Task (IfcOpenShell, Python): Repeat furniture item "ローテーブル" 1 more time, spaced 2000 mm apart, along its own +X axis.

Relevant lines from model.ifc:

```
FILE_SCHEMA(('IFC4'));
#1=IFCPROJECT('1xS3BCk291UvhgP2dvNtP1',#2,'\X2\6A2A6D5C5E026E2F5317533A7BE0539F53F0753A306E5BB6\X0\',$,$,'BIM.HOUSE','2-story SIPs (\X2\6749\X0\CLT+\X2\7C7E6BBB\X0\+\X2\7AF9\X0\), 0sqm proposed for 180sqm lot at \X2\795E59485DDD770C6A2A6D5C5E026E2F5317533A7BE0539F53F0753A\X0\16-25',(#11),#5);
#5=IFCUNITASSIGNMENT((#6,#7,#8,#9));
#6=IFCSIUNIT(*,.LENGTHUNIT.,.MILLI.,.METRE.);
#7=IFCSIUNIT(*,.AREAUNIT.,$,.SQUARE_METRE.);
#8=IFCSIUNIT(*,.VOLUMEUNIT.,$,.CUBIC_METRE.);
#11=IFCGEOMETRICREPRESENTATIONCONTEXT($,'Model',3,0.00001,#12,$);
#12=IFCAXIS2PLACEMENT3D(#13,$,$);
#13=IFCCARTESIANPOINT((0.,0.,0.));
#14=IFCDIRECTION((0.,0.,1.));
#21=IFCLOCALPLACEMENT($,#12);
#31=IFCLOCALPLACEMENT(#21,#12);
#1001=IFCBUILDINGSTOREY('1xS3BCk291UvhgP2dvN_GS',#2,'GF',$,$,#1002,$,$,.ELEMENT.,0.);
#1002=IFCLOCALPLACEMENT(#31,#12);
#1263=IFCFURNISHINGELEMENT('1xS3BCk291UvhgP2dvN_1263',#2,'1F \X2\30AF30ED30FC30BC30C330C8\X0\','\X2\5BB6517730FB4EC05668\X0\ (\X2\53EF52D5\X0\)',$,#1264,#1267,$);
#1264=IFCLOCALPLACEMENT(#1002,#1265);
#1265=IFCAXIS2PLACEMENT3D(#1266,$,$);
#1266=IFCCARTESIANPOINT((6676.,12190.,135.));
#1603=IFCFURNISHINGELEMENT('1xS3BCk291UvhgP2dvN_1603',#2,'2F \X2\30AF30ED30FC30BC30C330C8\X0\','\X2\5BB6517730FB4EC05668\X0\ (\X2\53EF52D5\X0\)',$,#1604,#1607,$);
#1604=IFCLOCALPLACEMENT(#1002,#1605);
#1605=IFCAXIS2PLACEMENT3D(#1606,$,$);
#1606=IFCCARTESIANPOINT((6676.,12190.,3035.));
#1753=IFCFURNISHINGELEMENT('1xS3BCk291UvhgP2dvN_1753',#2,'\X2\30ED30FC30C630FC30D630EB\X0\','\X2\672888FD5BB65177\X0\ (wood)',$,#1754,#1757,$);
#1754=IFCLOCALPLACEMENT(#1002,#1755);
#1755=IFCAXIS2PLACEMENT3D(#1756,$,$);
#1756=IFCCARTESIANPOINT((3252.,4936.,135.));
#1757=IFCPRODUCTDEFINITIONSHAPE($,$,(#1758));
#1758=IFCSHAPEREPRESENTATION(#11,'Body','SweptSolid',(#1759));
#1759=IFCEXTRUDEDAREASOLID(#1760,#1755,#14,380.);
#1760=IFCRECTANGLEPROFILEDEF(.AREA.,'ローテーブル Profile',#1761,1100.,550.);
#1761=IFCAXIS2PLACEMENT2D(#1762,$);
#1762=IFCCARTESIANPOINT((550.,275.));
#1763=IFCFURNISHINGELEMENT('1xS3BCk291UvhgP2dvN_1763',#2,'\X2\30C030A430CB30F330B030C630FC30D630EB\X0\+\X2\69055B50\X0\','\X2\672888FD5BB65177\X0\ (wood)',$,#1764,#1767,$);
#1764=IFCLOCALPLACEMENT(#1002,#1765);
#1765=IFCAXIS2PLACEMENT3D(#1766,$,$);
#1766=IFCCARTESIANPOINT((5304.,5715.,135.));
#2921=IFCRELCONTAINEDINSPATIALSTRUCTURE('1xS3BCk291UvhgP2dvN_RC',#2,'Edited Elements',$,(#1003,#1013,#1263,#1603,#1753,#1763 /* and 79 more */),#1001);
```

```python
import ifcopenshell
import ifcopenshell.api.geometry
import ifcopenshell.api.root
import ifcopenshell.util.element
import ifcopenshell.util.placement
import ifcopenshell.util.unit

model = ifcopenshell.open("model.ifc")
unit_scale = ifcopenshell.util.unit.calculate_unit_scale(model)


def reuse_history(source, copy):
    """copy_class also copies each property set's owner history, people and application; keep the originals."""
    for rel in copy.IsDefinedBy:
        if rel.is_a("IfcRelDefinesByProperties") and (history := rel.RelatingPropertyDefinition.OwnerHistory):
            rel.RelatingPropertyDefinition.OwnerHistory = source.OwnerHistory
            ifcopenshell.util.element.remove_deep2(model, history)


source = model.by_id(1753)
base = ifcopenshell.util.placement.get_local_placement(source.ObjectPlacement)
step = base[:3, 0] * 2 / unit_scale

for i in range(1, 2):
    copy = ifcopenshell.api.root.copy_class(model, product=source)
    copy.Representation = ifcopenshell.util.element.copy_deep(
        model, source.Representation, exclude=["IfcGeometricRepresentationContext", "IfcRepresentationMap"]
    )
    reuse_history(source, copy)
    matrix = base.copy()
    matrix[:3, 3] += i * step
    print("added at", matrix[:3, 3].round(3) + 0.0)
    ifcopenshell.api.geometry.edit_object_placement(model, product=copy, matrix=matrix, is_si=False)

model.write("model_v2.ifc")
```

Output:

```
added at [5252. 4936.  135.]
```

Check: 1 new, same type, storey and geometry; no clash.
